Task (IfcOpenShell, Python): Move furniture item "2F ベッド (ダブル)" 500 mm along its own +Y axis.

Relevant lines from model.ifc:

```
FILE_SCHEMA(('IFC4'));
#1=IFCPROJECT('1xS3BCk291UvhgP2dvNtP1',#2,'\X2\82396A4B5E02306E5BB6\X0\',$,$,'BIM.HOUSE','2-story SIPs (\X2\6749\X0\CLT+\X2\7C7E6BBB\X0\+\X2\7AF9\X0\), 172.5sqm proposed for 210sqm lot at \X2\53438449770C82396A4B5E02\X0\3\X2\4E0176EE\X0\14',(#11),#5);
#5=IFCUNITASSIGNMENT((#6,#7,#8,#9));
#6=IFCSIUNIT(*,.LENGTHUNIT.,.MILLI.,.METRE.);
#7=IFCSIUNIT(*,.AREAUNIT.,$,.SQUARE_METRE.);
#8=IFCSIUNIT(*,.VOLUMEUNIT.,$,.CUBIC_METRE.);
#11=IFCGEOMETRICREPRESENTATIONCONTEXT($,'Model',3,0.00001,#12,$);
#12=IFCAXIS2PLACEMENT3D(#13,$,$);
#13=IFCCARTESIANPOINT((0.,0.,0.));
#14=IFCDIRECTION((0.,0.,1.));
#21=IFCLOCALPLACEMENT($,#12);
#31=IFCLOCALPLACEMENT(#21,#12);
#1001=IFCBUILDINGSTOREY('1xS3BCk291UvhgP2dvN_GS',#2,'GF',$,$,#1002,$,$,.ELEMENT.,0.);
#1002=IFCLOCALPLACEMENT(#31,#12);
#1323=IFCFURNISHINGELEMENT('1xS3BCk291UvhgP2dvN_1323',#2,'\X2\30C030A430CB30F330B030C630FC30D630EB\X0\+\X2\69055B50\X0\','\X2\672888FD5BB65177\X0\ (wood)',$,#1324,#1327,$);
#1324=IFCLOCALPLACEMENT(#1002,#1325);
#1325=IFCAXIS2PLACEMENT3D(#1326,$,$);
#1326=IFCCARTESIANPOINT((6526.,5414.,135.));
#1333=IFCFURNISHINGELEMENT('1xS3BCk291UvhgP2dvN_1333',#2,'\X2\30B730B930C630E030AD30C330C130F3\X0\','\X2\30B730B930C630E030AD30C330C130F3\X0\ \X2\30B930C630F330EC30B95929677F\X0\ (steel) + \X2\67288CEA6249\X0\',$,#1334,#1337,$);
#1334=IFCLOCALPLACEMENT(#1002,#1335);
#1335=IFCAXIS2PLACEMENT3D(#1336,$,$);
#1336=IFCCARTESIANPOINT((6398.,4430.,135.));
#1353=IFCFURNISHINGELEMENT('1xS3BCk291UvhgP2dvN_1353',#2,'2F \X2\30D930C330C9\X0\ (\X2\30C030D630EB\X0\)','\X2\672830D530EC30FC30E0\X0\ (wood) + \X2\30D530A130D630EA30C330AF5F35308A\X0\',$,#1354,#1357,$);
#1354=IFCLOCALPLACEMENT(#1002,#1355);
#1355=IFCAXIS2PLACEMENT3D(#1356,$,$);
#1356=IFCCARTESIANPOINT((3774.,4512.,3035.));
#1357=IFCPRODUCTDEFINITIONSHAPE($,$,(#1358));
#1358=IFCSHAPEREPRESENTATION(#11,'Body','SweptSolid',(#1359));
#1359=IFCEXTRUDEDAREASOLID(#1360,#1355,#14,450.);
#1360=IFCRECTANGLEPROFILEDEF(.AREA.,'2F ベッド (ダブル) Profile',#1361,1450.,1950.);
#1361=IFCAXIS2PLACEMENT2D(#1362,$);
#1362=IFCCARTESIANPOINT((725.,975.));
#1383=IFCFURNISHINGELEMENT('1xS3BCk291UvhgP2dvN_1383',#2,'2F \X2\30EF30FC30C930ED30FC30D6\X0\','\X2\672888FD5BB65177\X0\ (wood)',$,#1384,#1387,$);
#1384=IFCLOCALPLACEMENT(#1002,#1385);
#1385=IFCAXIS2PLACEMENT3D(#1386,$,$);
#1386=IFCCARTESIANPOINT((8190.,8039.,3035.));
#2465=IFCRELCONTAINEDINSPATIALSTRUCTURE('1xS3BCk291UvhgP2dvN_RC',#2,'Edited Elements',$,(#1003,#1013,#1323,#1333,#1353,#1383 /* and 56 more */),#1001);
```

```python
import ifcopenshell
import ifcopenshell.api.geometry
import ifcopenshell.util.placement

model = ifcopenshell.open("model.ifc")

item = model.by_guid("1xS3BCk291UvhgP2dvN_1353")
matrix = ifcopenshell.util.placement.get_local_placement(item.ObjectPlacement)
matrix[:3, 3] += matrix[:3, 1] * 500.0
ifcopenshell.api.geometry.edit_object_placement(model, product=item, matrix=matrix, is_si=False)

print(ifcopenshell.util.placement.get_local_placement(item.ObjectPlacement).round(3) + 0.0)

model.write("model_edited.ifc")
```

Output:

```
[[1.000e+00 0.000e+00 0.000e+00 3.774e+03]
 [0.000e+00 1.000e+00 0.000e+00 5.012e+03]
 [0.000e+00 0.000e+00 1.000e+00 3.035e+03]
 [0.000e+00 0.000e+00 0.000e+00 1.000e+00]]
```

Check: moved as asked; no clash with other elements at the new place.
